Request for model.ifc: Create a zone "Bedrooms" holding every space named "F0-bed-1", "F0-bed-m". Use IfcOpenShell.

First a look at what the model holds.

```python
import ifcopenshell

model = ifcopenshell.open("model.ifc")
print(model.schema)
seen = {}
for space in model.by_type("IfcSpace"):
    seen[space.LongName] = seen.get(space.LongName, 0) + 1
for name, count in sorted(seen.items(), key=str):
    print(count, "x", name)
print("zones:", [z.Name for z in model.by_type("IfcZone")][:20])
```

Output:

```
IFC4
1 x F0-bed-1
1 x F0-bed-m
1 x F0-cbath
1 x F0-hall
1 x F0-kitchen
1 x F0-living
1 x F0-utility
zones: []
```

```python
import ifcopenshell
import ifcopenshell.api.group
import ifcopenshell.api.root

model = ifcopenshell.open("model.ifc")

names = {"F0-bed-1", "F0-bed-m"}
spaces = [s for s in model.by_type("IfcSpace") if s.LongName in names]

zone = ifcopenshell.api.root.create_entity(model, ifc_class="IfcZone", name="Bedrooms")
ifcopenshell.api.group.assign_group(model, products=spaces, group=zone)
print(len(spaces), "spaces in", zone.Name)

model.write("model_edited.ifc")
```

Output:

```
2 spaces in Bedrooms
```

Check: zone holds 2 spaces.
